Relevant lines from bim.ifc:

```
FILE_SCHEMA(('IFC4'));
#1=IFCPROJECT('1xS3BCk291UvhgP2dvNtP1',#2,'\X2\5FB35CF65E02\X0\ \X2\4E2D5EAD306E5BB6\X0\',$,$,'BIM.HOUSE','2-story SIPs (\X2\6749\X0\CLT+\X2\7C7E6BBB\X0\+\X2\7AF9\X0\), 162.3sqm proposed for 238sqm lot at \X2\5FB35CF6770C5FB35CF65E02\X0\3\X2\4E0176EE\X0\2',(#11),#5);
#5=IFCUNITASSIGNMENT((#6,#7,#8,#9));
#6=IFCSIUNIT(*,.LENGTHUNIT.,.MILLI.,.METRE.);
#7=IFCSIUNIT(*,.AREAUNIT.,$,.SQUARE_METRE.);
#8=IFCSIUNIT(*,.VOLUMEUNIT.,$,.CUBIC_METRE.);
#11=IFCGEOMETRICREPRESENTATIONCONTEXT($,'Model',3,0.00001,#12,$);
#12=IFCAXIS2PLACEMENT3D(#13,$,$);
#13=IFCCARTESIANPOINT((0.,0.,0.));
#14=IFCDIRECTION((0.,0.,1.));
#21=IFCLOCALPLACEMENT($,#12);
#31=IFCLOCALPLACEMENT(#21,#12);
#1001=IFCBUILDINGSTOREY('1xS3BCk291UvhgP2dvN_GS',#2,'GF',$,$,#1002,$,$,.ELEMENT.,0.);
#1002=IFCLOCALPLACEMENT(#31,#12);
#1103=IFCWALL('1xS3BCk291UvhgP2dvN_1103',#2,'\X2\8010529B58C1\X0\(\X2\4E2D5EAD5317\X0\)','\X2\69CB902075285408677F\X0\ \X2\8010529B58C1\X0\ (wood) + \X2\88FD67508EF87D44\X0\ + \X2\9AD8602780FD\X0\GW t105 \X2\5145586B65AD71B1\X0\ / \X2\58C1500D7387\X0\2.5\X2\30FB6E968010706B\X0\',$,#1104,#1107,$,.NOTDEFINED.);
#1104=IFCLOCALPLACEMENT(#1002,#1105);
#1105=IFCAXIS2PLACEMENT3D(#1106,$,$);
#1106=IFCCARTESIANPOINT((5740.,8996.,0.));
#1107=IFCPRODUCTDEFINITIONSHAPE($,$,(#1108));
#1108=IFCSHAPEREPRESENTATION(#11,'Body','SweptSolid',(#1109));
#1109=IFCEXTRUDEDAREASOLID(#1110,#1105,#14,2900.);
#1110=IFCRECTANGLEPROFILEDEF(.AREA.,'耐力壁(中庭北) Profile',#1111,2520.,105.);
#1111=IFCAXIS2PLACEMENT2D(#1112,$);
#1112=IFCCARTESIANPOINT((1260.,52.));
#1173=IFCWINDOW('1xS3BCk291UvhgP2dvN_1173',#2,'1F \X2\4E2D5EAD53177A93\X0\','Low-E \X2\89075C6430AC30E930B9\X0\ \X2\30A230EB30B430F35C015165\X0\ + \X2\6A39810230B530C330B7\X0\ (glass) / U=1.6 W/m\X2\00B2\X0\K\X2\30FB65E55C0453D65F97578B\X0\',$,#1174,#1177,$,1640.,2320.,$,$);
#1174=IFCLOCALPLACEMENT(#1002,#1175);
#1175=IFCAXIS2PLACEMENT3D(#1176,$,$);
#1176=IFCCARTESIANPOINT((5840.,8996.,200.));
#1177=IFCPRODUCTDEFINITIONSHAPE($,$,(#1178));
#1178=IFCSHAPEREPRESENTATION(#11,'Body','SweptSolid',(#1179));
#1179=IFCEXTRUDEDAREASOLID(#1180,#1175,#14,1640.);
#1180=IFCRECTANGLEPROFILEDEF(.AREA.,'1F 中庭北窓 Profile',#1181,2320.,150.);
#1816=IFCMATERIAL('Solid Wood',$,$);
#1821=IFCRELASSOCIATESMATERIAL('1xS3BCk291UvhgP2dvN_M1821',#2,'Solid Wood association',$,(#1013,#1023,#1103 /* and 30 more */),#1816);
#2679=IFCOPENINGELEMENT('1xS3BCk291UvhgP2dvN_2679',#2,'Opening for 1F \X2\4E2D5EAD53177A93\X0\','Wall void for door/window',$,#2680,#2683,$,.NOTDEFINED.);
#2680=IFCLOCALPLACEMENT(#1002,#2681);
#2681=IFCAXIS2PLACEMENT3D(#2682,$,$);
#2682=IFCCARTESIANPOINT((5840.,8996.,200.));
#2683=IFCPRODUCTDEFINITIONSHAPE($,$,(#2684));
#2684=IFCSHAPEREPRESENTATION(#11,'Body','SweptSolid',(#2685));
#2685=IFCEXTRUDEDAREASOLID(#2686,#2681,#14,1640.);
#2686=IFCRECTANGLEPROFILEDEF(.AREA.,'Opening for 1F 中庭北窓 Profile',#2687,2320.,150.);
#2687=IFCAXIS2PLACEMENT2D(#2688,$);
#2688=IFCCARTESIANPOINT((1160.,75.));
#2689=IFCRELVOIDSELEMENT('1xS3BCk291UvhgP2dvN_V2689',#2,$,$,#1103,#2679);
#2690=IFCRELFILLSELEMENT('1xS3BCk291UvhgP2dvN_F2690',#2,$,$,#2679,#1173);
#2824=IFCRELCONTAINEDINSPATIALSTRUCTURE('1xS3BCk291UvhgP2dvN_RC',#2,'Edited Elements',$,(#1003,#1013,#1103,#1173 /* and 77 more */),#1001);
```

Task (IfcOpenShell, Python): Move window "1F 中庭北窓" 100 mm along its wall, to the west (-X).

```python
import ifcopenshell
import ifcopenshell.api.geometry
import ifcopenshell.util.placement

model = ifcopenshell.open("bim.ifc")

window = model.by_id(1173)
opening = window.FillsVoids[0].RelatingOpeningElement
wall = opening.VoidsElements[0].RelatingBuildingElement

wall_matrix = ifcopenshell.util.placement.get_local_placement(wall.ObjectPlacement)
shift = wall_matrix[:3, 0] * -100.0
before = ifcopenshell.util.placement.get_local_placement(window.ObjectPlacement)[:3, 3].copy()

# The window is not placed relative to its opening, so move both.
for product in (opening, window):
    matrix = ifcopenshell.util.placement.get_local_placement(product.ObjectPlacement)
    matrix[:3, 3] += shift
    ifcopenshell.api.geometry.edit_object_placement(model, product=product, matrix=matrix, is_si=False)

after = ifcopenshell.util.placement.get_local_placement(window.ObjectPlacement)[:3, 3]
print("window moved by", (after - before).round(3) + 0.0)

model.write("bim_rev.ifc")
```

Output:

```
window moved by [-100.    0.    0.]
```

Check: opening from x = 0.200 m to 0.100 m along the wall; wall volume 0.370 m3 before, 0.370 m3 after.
